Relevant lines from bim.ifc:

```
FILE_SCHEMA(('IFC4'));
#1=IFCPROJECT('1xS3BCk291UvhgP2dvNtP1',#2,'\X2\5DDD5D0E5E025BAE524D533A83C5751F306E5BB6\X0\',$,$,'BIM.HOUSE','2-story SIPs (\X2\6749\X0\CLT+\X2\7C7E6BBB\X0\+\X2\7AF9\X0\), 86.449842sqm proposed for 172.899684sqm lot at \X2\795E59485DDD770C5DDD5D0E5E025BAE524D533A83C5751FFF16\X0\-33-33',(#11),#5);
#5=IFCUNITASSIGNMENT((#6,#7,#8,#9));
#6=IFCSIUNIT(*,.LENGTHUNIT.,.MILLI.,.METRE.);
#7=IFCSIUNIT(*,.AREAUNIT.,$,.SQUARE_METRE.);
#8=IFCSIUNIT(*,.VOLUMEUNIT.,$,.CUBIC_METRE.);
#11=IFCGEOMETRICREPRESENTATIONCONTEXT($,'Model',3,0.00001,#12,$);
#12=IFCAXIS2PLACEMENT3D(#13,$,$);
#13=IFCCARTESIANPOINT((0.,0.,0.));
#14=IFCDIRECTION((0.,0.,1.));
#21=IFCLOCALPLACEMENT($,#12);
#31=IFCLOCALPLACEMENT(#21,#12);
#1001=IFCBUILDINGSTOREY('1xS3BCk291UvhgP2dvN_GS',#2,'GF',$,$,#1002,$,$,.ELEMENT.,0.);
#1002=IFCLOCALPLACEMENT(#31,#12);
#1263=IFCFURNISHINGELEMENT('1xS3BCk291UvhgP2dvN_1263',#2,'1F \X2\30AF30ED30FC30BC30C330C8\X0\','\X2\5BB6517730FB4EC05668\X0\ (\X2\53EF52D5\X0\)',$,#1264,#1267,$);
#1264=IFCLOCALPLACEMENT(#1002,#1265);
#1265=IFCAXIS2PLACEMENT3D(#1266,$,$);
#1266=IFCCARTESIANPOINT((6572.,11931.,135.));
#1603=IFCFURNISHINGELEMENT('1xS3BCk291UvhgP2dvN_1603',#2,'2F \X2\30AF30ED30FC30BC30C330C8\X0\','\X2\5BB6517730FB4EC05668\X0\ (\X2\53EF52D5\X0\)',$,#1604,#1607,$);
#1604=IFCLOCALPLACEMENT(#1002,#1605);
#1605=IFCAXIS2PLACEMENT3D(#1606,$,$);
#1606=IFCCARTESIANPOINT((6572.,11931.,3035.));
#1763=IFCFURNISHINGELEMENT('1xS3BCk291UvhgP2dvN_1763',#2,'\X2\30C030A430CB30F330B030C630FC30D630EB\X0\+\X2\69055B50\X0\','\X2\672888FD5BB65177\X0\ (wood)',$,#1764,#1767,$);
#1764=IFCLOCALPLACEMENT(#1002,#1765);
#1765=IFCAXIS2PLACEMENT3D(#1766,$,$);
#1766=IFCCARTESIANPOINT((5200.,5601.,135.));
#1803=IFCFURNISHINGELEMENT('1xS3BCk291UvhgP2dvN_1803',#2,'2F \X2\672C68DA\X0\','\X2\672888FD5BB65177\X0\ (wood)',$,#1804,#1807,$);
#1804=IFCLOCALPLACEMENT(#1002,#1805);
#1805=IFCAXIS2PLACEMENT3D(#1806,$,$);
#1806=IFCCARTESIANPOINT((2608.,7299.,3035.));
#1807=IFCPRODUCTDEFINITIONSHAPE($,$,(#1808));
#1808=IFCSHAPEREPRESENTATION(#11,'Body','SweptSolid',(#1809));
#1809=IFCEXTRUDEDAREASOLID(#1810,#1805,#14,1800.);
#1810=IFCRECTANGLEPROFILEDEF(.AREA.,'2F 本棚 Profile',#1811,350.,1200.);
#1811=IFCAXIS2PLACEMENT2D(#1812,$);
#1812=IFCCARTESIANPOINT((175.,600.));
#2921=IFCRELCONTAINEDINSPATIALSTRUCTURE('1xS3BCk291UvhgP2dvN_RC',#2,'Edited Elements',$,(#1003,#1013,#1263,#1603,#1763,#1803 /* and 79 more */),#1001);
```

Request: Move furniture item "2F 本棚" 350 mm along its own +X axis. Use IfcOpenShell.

```python
import ifcopenshell
import ifcopenshell.api.geometry
import ifcopenshell.util.placement

model = ifcopenshell.open("bim.ifc")

item = model.by_guid("1xS3BCk291UvhgP2dvN_1803")
matrix = ifcopenshell.util.placement.get_local_placement(item.ObjectPlacement)
matrix[:3, 3] += matrix[:3, 0] * 350.0
ifcopenshell.api.geometry.edit_object_placement(model, product=item, matrix=matrix, is_si=False)

print(ifcopenshell.util.placement.get_local_placement(item.ObjectPlacement).round(3) + 0.0)

model.write("bim_rev.ifc")
```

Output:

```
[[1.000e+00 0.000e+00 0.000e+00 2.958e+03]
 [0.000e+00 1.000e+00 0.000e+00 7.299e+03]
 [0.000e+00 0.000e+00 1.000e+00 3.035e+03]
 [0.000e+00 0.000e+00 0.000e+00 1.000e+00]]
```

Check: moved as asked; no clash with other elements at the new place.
